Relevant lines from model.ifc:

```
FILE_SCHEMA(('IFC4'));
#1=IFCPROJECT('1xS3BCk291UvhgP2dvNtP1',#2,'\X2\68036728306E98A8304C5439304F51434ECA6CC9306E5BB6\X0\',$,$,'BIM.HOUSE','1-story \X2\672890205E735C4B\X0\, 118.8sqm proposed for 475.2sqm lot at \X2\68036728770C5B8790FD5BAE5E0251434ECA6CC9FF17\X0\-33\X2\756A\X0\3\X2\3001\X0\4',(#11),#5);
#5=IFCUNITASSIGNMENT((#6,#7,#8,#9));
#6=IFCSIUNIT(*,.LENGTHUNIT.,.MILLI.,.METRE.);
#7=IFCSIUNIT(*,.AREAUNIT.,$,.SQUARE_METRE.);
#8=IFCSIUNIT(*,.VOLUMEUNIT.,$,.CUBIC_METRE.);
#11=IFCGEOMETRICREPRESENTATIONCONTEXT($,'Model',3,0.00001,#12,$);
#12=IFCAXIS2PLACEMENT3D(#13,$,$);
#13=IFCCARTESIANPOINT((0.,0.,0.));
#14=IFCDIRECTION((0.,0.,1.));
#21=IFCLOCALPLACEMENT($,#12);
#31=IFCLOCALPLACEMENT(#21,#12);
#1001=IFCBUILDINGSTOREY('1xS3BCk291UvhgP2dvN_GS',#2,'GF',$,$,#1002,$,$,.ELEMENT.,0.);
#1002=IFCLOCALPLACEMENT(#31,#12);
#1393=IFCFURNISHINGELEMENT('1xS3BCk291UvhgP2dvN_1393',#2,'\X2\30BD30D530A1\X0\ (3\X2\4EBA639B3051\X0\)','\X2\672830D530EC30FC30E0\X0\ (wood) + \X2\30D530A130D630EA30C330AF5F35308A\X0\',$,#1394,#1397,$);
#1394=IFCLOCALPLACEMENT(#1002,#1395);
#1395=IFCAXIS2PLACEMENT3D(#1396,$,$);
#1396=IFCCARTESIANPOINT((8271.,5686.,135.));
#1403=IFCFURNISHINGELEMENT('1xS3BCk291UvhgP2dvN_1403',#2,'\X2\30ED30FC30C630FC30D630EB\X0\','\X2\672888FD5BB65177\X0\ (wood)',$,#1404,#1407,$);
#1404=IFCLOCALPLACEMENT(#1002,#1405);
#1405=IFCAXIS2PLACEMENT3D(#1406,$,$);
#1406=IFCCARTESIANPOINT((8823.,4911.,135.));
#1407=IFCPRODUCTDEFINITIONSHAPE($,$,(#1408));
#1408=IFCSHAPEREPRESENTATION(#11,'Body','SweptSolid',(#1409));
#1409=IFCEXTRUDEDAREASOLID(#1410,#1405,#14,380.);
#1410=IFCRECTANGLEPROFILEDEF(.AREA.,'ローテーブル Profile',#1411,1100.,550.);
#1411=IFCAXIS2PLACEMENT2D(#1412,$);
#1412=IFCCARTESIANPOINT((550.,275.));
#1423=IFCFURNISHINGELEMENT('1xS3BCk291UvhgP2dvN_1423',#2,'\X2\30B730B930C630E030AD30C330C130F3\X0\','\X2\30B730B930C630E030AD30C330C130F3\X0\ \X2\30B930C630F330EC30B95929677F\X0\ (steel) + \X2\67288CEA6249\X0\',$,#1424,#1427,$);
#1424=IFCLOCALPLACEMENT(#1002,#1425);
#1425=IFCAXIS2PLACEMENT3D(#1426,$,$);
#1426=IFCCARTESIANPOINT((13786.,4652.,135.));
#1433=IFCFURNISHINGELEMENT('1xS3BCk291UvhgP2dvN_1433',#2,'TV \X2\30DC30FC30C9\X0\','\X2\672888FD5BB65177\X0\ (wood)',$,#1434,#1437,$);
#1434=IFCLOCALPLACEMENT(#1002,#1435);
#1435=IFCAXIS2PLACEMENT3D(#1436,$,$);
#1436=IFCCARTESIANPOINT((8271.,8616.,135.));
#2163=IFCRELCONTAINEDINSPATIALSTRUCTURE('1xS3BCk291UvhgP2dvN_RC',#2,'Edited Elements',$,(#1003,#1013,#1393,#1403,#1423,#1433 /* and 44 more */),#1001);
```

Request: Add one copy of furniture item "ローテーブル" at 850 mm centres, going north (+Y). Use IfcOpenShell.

```python
import numpy as np
import ifcopenshell
import ifcopenshell.api.geometry
import ifcopenshell.api.root
import ifcopenshell.util.element
import ifcopenshell.util.placement
import ifcopenshell.util.unit

model = ifcopenshell.open("model.ifc")
unit_scale = ifcopenshell.util.unit.calculate_unit_scale(model)


def reuse_history(source, copy):
    """copy_class also copies each property set's owner history, people and application; keep the originals."""
    for rel in copy.IsDefinedBy:
        if rel.is_a("IfcRelDefinesByProperties") and (history := rel.RelatingPropertyDefinition.OwnerHistory):
            rel.RelatingPropertyDefinition.OwnerHistory = source.OwnerHistory
            ifcopenshell.util.element.remove_deep2(model, history)


source = model.by_id(1403)
base = ifcopenshell.util.placement.get_local_placement(source.ObjectPlacement)
step = np.array([0.0, 1.0, 0.0]) * 0.85 / unit_scale

for i in range(1, 2):
    copy = ifcopenshell.api.root.copy_class(model, product=source)
    copy.Representation = ifcopenshell.util.element.copy_deep(
        model, source.Representation, exclude=["IfcGeometricRepresentationContext", "IfcRepresentationMap"]
    )
    reuse_history(source, copy)
    matrix = base.copy()
    matrix[:3, 3] += i * step
    print("added at", matrix[:3, 3].round(3) + 0.0)
    ifcopenshell.api.geometry.edit_object_placement(model, product=copy, matrix=matrix, is_si=False)

model.write("model_v2.ifc")
```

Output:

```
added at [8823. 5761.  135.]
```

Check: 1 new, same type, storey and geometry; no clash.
